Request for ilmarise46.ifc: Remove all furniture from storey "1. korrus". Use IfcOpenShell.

First a look at what the model holds.

```python
import ifcopenshell
import ifcopenshell.util.element

model = ifcopenshell.open("ilmarise46.ifc")
print(model.schema)
storey = next(s for s in model.by_type("IfcBuildingStorey") if s.Name == "1. korrus")
furniture = [e for e in ifcopenshell.util.element.get_decomposition(storey) if e.is_a("IfcFurnishingElement")]
seen = {}
for e in furniture:
    element_type = ifcopenshell.util.element.get_type(e)
    name = element_type.Name if element_type not in (None, e) else None
    seen[name] = seen.get(name, 0) + 1
for name, count in sorted(seen.items(), key=str):
    print(count, "x", name)
```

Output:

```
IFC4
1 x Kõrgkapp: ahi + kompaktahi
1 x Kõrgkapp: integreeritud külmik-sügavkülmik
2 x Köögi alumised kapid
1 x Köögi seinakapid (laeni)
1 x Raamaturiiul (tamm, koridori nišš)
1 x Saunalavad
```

```python
import ifcopenshell
import ifcopenshell.api.root
import ifcopenshell.util.element

model = ifcopenshell.open("ilmarise46.ifc")

storey = next(s for s in model.by_type("IfcBuildingStorey") if s.Name == "1. korrus")
furniture = [e for e in ifcopenshell.util.element.get_decomposition(storey) if e.is_a("IfcFurnishingElement")]

for e in furniture:
    ifcopenshell.api.root.remove_product(model, product=e)
print(len(furniture), "removed")

model.write("ilmarise46_edited.ifc")
```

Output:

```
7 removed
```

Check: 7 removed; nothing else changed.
